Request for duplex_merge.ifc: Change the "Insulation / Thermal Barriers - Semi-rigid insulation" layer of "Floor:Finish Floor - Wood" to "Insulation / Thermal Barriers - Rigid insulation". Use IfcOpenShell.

First a look at what the model holds.

```python
import ifcopenshell
import ifcopenshell.util.element

model = ifcopenshell.open("duplex_merge.ifc")
print(model.schema)
for layer_set in model.by_type("IfcMaterialLayerSet"):
    if layer_set.LayerSetName == "Floor:Finish Floor - Wood":
        for layer in layer_set.MaterialLayers:
            print(layer.id(), layer.Material and layer.Material.Name, layer.LayerThickness, sep=" | ")
        print(len(ifcopenshell.util.element.get_elements_by_material(model, layer_set)), "elements and types use it")
print(sorted(m.Name for m in model.by_type("IfcMaterial") if m.Name)[:60])
```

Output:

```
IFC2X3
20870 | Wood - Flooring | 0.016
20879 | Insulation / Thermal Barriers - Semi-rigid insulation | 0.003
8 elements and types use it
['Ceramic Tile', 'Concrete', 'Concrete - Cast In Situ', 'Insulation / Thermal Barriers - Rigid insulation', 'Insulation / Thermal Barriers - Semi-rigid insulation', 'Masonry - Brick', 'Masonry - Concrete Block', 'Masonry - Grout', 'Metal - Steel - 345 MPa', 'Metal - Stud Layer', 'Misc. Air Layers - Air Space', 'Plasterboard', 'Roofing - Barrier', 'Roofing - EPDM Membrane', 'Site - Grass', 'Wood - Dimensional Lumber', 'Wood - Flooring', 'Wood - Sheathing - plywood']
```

```python
import ifcopenshell
import ifcopenshell.api.material

model = ifcopenshell.open("duplex_merge.ifc")

layer_set = next(s for s in model.by_type("IfcMaterialLayerSet") if s.LayerSetName == "Floor:Finish Floor - Wood")
layer = next(l for l in layer_set.MaterialLayers if l.Material and l.Material.Name == "Insulation / Thermal Barriers - Semi-rigid insulation")
material = next(m for m in model.by_type("IfcMaterial") if m.Name == "Insulation / Thermal Barriers - Rigid insulation")

# Point this one layer at the other material; renaming the old one would change it everywhere.
ifcopenshell.api.material.edit_layer(model, layer=layer, attributes={}, material=material)

print([l.Material.Name if l.Material else None for l in layer_set.MaterialLayers])

model.write("duplex_merge_v2.ifc")
```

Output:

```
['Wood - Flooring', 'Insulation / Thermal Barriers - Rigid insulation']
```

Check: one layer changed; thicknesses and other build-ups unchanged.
